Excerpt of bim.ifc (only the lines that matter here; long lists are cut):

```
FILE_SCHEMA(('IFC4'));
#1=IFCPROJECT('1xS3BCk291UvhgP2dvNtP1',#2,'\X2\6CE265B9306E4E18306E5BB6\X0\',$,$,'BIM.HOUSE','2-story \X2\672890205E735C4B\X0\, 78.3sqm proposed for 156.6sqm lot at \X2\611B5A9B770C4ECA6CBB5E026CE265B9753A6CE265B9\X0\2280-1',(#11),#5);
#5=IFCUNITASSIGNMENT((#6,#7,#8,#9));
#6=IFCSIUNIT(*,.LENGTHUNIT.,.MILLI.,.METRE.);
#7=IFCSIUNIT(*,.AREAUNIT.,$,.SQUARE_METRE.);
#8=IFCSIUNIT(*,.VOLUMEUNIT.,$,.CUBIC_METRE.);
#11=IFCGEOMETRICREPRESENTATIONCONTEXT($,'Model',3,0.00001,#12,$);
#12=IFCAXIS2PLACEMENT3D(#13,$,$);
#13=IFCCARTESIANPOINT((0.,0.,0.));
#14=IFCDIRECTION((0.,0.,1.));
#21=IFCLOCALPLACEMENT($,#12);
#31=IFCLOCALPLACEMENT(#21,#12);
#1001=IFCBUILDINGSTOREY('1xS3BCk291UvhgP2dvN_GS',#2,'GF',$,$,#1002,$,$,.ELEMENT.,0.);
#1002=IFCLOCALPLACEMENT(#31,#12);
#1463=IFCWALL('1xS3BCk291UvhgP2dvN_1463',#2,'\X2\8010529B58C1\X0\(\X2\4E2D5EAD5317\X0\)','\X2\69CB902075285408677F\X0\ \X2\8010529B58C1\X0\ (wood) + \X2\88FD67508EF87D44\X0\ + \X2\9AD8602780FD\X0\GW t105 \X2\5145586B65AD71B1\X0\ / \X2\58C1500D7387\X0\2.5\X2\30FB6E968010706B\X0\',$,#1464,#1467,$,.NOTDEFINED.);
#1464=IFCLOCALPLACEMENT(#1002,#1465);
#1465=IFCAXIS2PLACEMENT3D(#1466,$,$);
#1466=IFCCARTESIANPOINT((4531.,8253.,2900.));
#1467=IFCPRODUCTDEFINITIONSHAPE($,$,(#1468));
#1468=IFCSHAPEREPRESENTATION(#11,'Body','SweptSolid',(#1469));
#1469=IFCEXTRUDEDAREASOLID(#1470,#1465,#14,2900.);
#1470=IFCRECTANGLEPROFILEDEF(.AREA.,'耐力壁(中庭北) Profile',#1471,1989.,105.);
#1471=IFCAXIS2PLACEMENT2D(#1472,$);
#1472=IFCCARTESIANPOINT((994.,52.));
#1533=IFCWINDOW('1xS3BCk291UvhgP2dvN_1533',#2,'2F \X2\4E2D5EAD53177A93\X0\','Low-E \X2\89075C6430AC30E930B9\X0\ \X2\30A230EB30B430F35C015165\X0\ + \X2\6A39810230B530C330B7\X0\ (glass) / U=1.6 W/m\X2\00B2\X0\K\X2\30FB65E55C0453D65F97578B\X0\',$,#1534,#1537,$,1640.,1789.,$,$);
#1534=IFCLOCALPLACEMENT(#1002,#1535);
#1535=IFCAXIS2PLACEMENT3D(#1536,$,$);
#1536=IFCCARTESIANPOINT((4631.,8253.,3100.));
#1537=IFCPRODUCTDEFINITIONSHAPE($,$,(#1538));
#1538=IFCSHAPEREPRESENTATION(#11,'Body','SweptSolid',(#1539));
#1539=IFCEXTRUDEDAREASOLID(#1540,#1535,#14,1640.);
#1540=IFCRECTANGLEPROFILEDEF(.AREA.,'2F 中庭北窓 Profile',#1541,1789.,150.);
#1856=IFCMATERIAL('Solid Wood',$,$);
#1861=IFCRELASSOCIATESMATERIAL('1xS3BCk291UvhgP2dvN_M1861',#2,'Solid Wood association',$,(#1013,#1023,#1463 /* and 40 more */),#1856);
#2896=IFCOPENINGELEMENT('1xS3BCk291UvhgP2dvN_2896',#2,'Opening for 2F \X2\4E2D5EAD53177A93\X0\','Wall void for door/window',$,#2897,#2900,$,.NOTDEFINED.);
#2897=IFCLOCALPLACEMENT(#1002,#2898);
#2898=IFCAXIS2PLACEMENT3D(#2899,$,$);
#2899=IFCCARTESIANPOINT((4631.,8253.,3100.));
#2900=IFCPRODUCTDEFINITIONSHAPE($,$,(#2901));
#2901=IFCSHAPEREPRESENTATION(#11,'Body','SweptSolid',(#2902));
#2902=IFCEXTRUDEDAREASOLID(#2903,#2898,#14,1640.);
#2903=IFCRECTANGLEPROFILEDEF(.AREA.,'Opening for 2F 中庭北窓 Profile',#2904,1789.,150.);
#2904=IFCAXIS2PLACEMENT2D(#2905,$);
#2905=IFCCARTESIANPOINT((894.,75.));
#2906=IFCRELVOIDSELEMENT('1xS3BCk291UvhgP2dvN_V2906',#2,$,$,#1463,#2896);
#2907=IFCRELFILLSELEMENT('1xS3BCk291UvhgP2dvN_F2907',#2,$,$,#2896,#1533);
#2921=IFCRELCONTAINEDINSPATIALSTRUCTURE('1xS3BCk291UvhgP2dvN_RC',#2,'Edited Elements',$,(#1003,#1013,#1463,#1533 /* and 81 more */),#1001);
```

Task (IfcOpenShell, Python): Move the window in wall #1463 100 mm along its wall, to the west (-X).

```python
import ifcopenshell
import ifcopenshell.api.geometry
import ifcopenshell.util.placement

model = ifcopenshell.open("bim.ifc")

window = model.by_guid("1xS3BCk291UvhgP2dvN_1533")
opening = window.FillsVoids[0].RelatingOpeningElement
wall = opening.VoidsElements[0].RelatingBuildingElement

wall_matrix = ifcopenshell.util.placement.get_local_placement(wall.ObjectPlacement)
shift = wall_matrix[:3, 0] * -100.0
before = ifcopenshell.util.placement.get_local_placement(window.ObjectPlacement)[:3, 3].copy()

# The window is not placed relative to its opening, so move both.
for product in (opening, window):
    matrix = ifcopenshell.util.placement.get_local_placement(product.ObjectPlacement)
    matrix[:3, 3] += shift
    ifcopenshell.api.geometry.edit_object_placement(model, product=product, matrix=matrix, is_si=False)

after = ifcopenshell.util.placement.get_local_placement(window.ObjectPlacement)[:3, 3]
print("window moved by", (after - before).round(3) + 0.0)

model.write("bim_edited.ifc")
```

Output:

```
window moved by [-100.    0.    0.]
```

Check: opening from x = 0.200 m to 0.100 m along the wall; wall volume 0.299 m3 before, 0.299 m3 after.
